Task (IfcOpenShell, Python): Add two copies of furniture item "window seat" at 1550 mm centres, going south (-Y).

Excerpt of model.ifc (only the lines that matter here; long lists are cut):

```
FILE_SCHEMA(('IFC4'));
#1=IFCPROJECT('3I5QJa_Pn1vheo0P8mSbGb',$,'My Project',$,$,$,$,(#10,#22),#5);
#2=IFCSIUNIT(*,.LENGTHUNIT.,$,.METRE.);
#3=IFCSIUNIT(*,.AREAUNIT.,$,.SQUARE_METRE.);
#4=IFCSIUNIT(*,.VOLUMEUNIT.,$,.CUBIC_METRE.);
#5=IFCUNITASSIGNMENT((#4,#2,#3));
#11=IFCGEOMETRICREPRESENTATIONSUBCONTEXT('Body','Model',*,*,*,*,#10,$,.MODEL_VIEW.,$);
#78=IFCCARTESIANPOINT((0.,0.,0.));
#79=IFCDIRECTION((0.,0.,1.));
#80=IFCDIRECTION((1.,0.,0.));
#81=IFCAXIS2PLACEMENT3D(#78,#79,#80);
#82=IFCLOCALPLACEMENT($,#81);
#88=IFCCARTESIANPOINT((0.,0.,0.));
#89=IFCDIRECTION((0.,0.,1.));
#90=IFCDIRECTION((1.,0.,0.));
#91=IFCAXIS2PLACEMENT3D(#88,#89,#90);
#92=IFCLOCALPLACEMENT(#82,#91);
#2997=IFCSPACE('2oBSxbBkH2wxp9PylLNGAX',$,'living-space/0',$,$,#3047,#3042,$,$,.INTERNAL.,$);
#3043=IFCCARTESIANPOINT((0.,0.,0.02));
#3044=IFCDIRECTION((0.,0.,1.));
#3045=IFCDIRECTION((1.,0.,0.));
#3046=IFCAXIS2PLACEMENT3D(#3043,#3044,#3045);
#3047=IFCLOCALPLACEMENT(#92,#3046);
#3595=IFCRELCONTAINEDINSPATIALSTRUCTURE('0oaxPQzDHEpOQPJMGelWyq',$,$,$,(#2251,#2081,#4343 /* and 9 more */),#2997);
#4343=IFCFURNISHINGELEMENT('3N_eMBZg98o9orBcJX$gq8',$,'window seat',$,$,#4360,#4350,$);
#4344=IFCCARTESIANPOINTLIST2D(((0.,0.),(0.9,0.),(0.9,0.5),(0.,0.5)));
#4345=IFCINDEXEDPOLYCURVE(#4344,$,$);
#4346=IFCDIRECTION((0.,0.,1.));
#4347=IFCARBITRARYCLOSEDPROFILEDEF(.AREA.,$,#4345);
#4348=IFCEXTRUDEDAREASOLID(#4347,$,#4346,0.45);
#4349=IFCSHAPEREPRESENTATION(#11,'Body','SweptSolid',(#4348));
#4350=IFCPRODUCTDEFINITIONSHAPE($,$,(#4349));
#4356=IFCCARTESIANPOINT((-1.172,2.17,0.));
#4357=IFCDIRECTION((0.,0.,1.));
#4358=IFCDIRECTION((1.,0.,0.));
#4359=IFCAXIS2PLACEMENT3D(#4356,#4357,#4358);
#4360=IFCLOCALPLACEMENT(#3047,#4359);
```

```python
import numpy as np
import ifcopenshell
import ifcopenshell.api.geometry
import ifcopenshell.api.root
import ifcopenshell.util.element
import ifcopenshell.util.placement
import ifcopenshell.util.unit

model = ifcopenshell.open("model.ifc")
unit_scale = ifcopenshell.util.unit.calculate_unit_scale(model)

source = model.by_id(4343)
base = ifcopenshell.util.placement.get_local_placement(source.ObjectPlacement)
step = np.array([0.0, -1.0, 0.0]) * 1.55 / unit_scale

for i in range(1, 3):
    copy = ifcopenshell.api.root.copy_class(model, product=source)
    copy.Representation = ifcopenshell.util.element.copy_deep(
        model, source.Representation, exclude=["IfcGeometricRepresentationContext", "IfcRepresentationMap"]
    )
    matrix = base.copy()
    matrix[:3, 3] += i * step
    print("added at", matrix[:3, 3].round(3) + 0.0)
    ifcopenshell.api.geometry.edit_object_placement(model, product=copy, matrix=matrix, is_si=False)

model.write("model_rev.ifc")
```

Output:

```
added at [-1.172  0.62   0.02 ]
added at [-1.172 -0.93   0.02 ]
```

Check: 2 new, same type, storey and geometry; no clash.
